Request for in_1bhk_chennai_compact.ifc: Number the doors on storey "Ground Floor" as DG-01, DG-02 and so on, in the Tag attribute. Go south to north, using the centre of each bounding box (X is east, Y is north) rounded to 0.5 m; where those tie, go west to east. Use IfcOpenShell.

First a look at what the model holds.

```python
import ifcopenshell
import ifcopenshell.util.element
import ifcopenshell.util.placement

model = ifcopenshell.open("in_1bhk_chennai_compact.ifc")
print(model.schema)
storey = next(s for s in model.by_type("IfcBuildingStorey") if s.Name == "Ground Floor")
doors = [e for e in ifcopenshell.util.element.get_decomposition(storey) if e.is_a("IfcDoor")]
for e in sorted(doors, key=lambda e: e.id()):
    origin = ifcopenshell.util.placement.get_local_placement(e.ObjectPlacement)[:3, 3]
    print(e.id(), e.Tag, e.Name, origin.round(2) + 0.0, sep=" | ")
```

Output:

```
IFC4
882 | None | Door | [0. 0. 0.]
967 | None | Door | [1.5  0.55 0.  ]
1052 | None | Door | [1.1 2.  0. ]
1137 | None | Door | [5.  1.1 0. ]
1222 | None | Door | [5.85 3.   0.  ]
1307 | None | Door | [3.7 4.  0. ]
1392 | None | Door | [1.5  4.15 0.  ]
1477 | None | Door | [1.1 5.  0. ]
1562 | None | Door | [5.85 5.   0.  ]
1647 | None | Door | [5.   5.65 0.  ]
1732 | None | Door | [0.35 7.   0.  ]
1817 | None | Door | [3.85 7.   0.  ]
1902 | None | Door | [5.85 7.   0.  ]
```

```python
import ifcopenshell
import ifcopenshell.geom
import ifcopenshell.util.element
import ifcopenshell.util.shape

model = ifcopenshell.open("in_1bhk_chennai_compact.ifc")
settings = ifcopenshell.geom.settings()
settings.set("use-world-coords", True)


def centre(element):
    shape = ifcopenshell.geom.create_shape(settings, element)
    return ifcopenshell.util.shape.get_bbox_centroid(shape.geometry)


storey = next(s for s in model.by_type("IfcBuildingStorey") if s.Name == "Ground Floor")
doors = [e for e in ifcopenshell.util.element.get_decomposition(storey) if e.is_a("IfcDoor")]

# Insertion points can sit at a corner or the storey origin, so sort by the geometry (in metres).
centres = {e: centre(e) for e in doors}
doors.sort(key=lambda e: (round(centres[e][1] / 0.5), centres[e][0]))

for i, e in enumerate(doors, start=1):
    number = f"DG-{i:02d}"
    e.Tag = number
    print(e.id(), number)

model.write("in_1bhk_chennai_compact_updated.ifc")
```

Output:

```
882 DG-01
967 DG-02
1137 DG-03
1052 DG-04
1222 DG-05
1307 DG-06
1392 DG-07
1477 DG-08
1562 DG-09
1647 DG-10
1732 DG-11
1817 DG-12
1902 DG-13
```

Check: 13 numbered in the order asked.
